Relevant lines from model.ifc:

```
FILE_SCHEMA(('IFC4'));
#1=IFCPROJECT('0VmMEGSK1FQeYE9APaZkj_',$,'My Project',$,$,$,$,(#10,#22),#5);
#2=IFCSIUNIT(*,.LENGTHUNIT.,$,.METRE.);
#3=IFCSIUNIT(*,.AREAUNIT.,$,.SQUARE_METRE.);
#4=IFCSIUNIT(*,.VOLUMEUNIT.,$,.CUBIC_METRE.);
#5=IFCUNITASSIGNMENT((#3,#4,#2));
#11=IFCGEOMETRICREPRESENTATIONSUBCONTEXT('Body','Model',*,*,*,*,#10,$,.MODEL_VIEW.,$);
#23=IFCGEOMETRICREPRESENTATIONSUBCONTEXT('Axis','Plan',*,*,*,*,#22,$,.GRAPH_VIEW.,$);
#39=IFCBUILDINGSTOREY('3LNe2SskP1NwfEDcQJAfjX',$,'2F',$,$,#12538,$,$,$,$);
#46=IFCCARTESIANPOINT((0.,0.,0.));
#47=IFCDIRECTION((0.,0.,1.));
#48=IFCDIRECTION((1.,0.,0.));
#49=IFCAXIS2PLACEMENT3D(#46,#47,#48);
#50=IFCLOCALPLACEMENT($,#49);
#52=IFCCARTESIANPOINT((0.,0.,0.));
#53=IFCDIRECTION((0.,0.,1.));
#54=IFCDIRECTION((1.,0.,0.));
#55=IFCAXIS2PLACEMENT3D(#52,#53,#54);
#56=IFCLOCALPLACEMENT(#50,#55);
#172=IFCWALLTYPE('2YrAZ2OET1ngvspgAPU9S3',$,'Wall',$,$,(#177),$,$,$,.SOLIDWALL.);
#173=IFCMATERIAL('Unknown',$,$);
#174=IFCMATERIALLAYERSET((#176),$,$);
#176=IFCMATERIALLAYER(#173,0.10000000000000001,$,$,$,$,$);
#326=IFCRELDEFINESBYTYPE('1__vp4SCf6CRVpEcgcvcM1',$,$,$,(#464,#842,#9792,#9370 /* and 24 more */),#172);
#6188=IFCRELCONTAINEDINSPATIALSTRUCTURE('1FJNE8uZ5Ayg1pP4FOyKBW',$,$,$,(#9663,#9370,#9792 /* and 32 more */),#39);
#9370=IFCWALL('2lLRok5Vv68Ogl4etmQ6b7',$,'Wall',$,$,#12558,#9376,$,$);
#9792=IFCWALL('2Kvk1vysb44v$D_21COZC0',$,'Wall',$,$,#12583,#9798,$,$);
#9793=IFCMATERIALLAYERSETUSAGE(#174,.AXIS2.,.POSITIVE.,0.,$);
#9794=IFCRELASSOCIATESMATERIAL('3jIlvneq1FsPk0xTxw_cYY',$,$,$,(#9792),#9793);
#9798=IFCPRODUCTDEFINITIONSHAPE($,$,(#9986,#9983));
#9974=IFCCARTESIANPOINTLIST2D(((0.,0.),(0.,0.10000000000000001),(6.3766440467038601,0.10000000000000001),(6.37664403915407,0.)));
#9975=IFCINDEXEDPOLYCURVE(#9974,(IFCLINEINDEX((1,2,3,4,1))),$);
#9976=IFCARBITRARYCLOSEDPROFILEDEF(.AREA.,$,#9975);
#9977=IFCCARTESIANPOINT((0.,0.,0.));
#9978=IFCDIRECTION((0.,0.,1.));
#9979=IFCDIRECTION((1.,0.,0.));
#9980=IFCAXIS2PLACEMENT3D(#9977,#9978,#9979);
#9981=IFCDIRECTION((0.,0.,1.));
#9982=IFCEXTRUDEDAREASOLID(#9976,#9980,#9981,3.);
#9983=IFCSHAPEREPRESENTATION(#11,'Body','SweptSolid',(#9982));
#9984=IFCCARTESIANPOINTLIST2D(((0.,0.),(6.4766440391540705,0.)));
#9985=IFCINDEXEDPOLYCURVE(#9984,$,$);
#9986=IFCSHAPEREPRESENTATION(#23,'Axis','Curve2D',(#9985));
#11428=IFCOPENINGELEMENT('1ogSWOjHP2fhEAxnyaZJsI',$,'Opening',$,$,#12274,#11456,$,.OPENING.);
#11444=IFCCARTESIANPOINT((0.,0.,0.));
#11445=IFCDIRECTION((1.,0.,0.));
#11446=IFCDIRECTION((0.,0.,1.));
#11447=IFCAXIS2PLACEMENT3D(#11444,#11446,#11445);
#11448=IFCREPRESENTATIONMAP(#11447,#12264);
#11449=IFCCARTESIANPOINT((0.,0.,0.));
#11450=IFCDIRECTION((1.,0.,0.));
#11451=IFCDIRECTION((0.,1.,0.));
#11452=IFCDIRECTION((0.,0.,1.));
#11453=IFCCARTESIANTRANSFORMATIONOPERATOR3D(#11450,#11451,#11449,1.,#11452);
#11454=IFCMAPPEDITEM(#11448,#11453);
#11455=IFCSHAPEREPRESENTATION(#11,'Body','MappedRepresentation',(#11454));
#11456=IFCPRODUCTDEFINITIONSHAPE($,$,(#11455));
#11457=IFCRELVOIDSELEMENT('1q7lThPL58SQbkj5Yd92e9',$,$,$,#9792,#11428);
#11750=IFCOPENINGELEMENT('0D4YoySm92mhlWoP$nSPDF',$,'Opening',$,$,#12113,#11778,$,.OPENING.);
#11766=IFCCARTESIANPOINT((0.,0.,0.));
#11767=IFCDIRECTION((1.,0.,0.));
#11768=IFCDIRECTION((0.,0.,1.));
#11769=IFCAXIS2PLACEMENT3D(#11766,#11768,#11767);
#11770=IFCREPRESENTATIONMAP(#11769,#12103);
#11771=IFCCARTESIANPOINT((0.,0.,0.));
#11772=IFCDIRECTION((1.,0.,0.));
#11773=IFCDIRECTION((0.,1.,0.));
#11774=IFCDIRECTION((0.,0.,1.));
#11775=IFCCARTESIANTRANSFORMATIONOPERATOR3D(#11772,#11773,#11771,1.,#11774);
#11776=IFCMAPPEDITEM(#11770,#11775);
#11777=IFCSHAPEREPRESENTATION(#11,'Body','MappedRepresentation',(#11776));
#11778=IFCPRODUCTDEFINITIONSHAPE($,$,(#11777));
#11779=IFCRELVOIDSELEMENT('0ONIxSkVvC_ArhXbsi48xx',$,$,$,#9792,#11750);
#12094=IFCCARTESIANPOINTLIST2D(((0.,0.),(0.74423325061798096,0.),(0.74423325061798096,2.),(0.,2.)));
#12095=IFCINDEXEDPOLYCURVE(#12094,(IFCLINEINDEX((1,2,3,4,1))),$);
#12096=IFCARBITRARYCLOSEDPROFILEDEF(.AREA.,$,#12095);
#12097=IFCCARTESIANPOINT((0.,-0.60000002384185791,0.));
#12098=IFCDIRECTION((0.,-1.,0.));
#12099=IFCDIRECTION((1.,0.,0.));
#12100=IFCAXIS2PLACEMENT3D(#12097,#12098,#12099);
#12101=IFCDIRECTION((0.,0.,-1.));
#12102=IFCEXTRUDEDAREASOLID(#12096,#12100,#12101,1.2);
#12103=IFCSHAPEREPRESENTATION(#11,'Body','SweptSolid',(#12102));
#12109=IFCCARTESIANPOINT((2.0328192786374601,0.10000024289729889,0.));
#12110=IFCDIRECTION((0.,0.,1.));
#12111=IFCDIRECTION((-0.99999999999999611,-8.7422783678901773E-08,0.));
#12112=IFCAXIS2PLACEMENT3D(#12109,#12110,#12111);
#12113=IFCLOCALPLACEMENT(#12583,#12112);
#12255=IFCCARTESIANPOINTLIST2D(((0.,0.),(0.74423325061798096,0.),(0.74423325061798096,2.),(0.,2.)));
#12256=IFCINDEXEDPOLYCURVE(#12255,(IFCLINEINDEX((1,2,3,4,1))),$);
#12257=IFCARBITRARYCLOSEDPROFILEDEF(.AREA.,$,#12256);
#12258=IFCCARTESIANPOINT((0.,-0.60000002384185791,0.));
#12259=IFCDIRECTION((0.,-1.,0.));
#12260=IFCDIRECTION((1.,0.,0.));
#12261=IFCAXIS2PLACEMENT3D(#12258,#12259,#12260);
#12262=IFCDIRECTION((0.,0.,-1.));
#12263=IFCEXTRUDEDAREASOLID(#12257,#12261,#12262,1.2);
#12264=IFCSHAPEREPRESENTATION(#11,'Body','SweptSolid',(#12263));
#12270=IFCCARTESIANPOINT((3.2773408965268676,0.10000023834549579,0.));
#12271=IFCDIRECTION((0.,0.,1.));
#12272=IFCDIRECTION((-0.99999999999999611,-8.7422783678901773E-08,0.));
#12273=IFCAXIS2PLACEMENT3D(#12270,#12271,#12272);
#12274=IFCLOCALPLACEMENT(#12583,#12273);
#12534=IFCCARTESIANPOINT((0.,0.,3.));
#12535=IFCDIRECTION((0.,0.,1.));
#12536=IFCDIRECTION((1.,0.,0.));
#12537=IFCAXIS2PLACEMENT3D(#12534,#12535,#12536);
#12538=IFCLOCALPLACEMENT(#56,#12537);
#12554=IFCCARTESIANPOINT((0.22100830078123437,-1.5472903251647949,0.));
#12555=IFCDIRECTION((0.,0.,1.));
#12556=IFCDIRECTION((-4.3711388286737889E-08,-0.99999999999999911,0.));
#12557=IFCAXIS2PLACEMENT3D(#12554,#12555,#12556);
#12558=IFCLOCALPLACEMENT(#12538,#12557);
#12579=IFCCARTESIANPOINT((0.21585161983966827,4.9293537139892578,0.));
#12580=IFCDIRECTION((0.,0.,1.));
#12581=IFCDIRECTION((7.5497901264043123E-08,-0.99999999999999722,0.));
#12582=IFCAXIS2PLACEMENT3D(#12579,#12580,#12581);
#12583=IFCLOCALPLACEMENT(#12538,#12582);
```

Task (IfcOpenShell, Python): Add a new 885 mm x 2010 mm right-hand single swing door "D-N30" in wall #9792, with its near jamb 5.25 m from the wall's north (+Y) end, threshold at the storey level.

```python
import numpy as np
import ifcopenshell
import ifcopenshell.api.feature
import ifcopenshell.api.geometry
import ifcopenshell.api.root
import ifcopenshell.api.spatial
import ifcopenshell.geom
import ifcopenshell.util.element
import ifcopenshell.util.placement
import ifcopenshell.util.representation
import ifcopenshell.util.shape
import ifcopenshell.util.unit

model = ifcopenshell.open("model.ifc")
unit_scale = ifcopenshell.util.unit.calculate_unit_scale(model)
settings = ifcopenshell.geom.settings()


def volume(element):
    """Net volume in cubic metres, openings subtracted."""
    shape = ifcopenshell.geom.create_shape(settings, element)
    return ifcopenshell.util.shape.get_volume(shape.geometry)


wall = model.by_guid("2Kvk1vysb44v$D_21COZC0")
storey = ifcopenshell.util.element.get_container(wall, ifc_class="IfcBuildingStorey")
context = ifcopenshell.util.representation.get_context(model, "Model", "Body", "MODEL_VIEW")
before = volume(wall)

width, height, from_end, sill = 0.885, 2.01, 5.25, 0.0  # metres

# The wall runs along its own X axis, and the end named is its -X end.
wall_shape = ifcopenshell.geom.create_shape(settings, wall)
x, y, z = ifcopenshell.util.shape.get_vertices(wall_shape.geometry).T
start = x.min() + from_end
face, thickness = float(y.min()), float(y.max() - y.min())
wall_matrix = ifcopenshell.util.placement.get_local_placement(wall.ObjectPlacement)
level = ifcopenshell.util.placement.get_local_placement(storey.ObjectPlacement)[2, 3]


def in_wall(x, y):
    """Placement at x, y metres in the wall's axes, at sill height."""
    matrix = wall_matrix.copy()
    matrix[:, 3] = wall_matrix @ np.array([x / unit_scale, y / unit_scale, 0.0, 1.0])
    matrix[2, 3] = level + sill / unit_scale
    return matrix


# Opening: a box that overshoots both wall faces by 50 mm.
opening = ifcopenshell.api.root.create_entity(model, ifc_class="IfcOpeningElement", predefined_type="OPENING")
box = ifcopenshell.api.geometry.add_wall_representation(
    model, context=context, length=width, height=height, thickness=thickness + 0.1
)
ifcopenshell.api.geometry.assign_representation(model, product=opening, representation=box)
ifcopenshell.api.geometry.edit_object_placement(model, product=opening, matrix=in_wall(start, face - 0.05), is_si=False)
ifcopenshell.api.feature.add_feature(model, feature=opening, element=wall)

door = ifcopenshell.api.root.create_entity(model, ifc_class="IfcDoor", name="D-N30", predefined_type="DOOR")
door.OverallWidth, door.OverallHeight = width / unit_scale, height / unit_scale
door.OperationType = "SINGLE_SWING_RIGHT"
body = ifcopenshell.api.geometry.add_door_representation(
    model,
    context=context,
    overall_width=door.OverallWidth,
    overall_height=door.OverallHeight,
    operation_type="SINGLE_SWING_RIGHT",
    lining_properties={"LiningDepth": thickness / unit_scale, "ThresholdDepth": thickness / unit_scale},
)
ifcopenshell.api.geometry.assign_representation(model, product=door, representation=body)
ifcopenshell.api.spatial.assign_container(model, products=[door], relating_structure=storey)
ifcopenshell.api.feature.add_filling(model, opening=opening, element=door)

# The lining spans the wall, so the door starts at the wall face.
ifcopenshell.api.geometry.edit_object_placement(model, product=door, matrix=in_wall(start, face), is_si=False)

after = volume(wall)

print(f"wall volume {before:.3f} -> {after:.3f} m3")

model.write("model_v2.ifc")
```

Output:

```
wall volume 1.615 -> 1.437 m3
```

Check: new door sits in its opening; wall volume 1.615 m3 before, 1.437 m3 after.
